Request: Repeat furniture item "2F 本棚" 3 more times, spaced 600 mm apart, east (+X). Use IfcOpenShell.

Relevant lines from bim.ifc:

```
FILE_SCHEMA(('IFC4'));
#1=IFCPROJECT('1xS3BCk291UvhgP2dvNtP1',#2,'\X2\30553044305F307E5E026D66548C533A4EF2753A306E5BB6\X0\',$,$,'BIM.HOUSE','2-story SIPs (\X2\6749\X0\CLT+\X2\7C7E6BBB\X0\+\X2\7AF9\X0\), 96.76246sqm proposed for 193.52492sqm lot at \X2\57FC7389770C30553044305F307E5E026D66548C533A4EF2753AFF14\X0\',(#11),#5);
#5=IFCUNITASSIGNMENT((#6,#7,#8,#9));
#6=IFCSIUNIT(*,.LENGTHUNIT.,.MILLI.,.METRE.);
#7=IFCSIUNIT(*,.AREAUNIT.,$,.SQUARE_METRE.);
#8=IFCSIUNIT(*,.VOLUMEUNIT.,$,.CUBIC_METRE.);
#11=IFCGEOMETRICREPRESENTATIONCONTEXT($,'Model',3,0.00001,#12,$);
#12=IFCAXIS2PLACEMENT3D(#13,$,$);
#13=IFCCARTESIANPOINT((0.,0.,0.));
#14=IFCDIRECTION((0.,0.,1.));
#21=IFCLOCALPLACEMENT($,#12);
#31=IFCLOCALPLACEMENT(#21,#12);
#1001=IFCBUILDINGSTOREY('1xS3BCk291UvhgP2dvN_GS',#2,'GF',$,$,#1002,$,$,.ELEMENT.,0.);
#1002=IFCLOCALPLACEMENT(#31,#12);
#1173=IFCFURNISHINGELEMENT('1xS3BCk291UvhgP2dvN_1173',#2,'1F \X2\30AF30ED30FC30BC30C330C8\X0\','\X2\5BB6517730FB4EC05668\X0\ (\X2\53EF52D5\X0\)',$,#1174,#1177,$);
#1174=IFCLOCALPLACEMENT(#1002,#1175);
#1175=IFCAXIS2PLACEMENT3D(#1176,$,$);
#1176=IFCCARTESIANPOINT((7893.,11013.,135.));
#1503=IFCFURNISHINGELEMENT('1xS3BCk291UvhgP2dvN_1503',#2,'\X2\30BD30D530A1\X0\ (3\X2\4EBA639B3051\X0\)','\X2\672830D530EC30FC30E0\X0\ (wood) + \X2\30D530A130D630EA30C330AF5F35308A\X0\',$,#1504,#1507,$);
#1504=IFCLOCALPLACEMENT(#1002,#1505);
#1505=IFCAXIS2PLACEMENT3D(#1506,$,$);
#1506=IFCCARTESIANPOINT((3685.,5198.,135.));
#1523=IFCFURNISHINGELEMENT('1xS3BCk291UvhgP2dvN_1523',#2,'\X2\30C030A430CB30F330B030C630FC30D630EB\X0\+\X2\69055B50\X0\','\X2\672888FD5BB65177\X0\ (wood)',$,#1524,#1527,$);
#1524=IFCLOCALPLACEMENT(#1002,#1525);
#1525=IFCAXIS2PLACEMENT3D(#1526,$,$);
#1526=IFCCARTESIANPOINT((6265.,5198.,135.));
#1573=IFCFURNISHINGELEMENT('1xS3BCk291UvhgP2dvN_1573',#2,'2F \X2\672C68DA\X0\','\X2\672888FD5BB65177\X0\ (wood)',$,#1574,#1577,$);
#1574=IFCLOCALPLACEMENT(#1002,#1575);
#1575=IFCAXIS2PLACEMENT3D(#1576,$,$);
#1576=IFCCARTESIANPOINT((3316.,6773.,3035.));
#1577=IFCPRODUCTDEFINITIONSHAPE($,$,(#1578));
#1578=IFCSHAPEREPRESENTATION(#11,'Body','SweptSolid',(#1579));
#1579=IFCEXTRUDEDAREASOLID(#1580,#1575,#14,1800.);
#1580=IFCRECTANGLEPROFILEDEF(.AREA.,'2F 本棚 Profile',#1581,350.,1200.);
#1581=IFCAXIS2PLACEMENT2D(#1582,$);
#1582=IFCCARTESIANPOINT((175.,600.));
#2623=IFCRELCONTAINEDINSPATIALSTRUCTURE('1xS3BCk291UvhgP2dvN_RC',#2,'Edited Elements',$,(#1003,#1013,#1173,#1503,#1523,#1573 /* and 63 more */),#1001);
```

```python
import numpy as np
import ifcopenshell
import ifcopenshell.api.geometry
import ifcopenshell.api.root
import ifcopenshell.util.element
import ifcopenshell.util.placement

model = ifcopenshell.open("bim.ifc")


def reuse_history(source, copy):
    """copy_class also copies each property set's owner history, people and application; keep the originals."""
    for rel in copy.IsDefinedBy:
        if rel.is_a("IfcRelDefinesByProperties") and (history := rel.RelatingPropertyDefinition.OwnerHistory):
            rel.RelatingPropertyDefinition.OwnerHistory = source.OwnerHistory
            ifcopenshell.util.element.remove_deep2(model, history)


source = model.by_guid("1xS3BCk291UvhgP2dvN_1573")
base = ifcopenshell.util.placement.get_local_placement(source.ObjectPlacement)
step = np.array([1.0, 0.0, 0.0]) * 600.0

for i in range(1, 4):
    copy = ifcopenshell.api.root.copy_class(model, product=source)
    copy.Representation = ifcopenshell.util.element.copy_deep(
        model, source.Representation, exclude=["IfcGeometricRepresentationContext", "IfcRepresentationMap"]
    )
    reuse_history(source, copy)
    matrix = base.copy()
    matrix[:3, 3] += i * step
    print("added at", matrix[:3, 3].round(3) + 0.0)
    ifcopenshell.api.geometry.edit_object_placement(model, product=copy, matrix=matrix, is_si=False)

model.write("bim_v2.ifc")
```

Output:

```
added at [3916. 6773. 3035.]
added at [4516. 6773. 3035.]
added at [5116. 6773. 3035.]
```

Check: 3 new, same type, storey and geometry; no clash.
